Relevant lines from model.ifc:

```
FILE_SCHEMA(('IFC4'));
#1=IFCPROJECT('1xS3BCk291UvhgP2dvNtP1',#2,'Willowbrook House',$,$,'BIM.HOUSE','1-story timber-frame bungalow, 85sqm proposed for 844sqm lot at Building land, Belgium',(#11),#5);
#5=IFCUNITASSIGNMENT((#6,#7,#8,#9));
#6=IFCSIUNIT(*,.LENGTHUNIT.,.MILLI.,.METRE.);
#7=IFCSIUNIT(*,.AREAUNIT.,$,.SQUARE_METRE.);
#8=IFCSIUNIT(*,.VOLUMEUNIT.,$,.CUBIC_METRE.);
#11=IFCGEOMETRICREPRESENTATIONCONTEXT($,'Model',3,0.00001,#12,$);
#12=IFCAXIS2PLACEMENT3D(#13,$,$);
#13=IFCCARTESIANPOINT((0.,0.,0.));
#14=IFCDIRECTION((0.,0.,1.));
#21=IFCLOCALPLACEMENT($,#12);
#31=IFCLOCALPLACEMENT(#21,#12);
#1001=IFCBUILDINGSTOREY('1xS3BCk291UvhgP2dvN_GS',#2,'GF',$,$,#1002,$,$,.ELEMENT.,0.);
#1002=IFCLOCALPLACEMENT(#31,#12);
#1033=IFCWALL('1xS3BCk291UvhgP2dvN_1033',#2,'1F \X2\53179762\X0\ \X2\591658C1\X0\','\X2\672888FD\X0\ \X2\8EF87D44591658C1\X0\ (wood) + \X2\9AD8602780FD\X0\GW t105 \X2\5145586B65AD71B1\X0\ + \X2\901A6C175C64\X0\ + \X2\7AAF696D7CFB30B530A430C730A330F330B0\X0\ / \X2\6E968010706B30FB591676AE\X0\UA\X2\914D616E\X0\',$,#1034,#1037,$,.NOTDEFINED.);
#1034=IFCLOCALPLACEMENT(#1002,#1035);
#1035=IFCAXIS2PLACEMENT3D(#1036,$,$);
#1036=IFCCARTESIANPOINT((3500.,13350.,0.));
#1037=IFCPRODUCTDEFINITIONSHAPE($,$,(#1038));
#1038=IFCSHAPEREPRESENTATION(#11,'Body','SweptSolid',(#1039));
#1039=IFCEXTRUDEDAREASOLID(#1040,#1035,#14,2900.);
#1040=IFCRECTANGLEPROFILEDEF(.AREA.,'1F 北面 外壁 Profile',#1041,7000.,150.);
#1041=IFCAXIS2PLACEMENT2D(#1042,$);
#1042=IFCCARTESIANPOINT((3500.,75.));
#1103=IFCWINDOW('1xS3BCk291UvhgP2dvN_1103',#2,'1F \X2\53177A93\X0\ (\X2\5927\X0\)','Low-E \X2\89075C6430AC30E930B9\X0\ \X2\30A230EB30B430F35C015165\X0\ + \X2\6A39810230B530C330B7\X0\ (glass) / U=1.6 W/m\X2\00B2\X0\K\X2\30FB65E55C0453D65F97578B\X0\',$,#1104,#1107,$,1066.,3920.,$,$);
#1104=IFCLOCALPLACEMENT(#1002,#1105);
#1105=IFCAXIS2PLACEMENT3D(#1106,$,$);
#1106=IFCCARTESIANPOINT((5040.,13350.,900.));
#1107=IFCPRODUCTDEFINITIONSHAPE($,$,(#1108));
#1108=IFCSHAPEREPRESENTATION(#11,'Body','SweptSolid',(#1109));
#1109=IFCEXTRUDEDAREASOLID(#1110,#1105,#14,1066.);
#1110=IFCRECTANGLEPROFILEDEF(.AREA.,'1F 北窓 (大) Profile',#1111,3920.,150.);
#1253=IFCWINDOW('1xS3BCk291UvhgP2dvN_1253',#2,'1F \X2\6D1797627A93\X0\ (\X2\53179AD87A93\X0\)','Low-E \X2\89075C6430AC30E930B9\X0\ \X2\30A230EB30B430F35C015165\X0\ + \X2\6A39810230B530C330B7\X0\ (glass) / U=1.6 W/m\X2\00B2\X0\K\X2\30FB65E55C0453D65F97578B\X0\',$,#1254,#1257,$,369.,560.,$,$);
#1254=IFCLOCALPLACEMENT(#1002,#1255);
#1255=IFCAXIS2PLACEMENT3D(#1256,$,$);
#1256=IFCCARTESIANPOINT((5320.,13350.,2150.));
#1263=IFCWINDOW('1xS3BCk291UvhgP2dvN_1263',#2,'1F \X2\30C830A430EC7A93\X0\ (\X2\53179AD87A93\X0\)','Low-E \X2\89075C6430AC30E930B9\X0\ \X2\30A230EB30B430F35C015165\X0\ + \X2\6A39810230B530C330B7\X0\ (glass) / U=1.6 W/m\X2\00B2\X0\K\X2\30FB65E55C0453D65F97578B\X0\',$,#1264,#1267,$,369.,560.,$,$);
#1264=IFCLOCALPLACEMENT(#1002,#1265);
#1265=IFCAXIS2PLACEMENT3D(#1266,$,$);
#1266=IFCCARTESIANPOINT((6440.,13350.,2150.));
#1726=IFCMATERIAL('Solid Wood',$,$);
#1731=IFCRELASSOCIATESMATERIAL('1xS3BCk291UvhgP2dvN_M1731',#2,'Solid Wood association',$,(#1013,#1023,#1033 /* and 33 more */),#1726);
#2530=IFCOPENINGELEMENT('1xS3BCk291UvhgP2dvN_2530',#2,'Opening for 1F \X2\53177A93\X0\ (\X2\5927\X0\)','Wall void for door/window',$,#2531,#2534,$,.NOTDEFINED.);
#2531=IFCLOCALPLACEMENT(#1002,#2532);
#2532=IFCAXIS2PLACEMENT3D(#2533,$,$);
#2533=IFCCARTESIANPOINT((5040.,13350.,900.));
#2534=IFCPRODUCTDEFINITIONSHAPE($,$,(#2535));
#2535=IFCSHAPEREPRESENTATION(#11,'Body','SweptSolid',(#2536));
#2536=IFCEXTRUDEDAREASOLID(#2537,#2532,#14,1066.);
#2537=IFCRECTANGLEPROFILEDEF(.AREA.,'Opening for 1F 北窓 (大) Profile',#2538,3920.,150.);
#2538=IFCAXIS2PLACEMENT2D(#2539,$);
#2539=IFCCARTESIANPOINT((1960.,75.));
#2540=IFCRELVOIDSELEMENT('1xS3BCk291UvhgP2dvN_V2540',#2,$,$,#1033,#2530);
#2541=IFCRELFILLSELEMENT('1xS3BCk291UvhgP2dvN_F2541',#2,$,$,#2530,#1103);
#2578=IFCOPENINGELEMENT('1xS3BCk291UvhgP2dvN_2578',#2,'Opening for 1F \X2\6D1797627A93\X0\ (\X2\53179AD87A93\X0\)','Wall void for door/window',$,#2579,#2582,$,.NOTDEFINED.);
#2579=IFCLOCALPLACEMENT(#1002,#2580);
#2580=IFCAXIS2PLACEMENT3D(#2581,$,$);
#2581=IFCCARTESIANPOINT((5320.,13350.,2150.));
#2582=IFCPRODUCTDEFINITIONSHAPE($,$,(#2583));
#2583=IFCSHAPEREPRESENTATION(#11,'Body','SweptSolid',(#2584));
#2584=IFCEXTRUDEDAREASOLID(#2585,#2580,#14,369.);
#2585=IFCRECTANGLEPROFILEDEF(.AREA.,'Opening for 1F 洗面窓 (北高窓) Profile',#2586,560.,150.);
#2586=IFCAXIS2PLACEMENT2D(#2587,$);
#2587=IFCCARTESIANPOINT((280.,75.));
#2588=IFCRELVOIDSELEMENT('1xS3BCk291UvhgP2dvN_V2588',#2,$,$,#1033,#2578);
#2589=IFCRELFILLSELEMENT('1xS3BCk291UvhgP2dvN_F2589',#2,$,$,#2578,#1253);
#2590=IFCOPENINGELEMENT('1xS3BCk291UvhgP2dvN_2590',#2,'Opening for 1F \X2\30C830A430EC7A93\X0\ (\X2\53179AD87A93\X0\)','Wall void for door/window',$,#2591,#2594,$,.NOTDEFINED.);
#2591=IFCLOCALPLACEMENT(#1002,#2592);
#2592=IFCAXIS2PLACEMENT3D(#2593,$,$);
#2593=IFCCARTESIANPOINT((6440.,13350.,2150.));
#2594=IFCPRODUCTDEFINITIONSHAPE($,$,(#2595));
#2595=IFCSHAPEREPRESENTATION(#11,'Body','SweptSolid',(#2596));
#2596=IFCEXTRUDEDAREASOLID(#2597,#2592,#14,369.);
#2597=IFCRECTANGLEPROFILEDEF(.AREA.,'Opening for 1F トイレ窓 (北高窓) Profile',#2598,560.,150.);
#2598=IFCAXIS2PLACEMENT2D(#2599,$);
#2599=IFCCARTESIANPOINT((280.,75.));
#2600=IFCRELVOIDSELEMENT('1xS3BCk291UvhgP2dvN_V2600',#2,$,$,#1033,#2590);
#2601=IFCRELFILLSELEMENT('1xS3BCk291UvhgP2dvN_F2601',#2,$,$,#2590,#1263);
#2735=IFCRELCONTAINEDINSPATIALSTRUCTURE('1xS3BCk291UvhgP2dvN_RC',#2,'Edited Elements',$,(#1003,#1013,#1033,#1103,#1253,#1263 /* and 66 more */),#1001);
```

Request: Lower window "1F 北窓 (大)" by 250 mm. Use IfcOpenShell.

```python
import numpy as np
import ifcopenshell
import ifcopenshell.api.geometry
import ifcopenshell.util.placement
import ifcopenshell.util.unit

model = ifcopenshell.open("model.ifc")
unit_scale = ifcopenshell.util.unit.calculate_unit_scale(model)

window = model.by_guid("1xS3BCk291UvhgP2dvN_1103")
opening = window.FillsVoids[0].RelatingOpeningElement
dz = -0.25 / unit_scale

shift = np.array([0.0, 0.0, dz])
# The window is not placed relative to its opening, so move both.
for product in (opening, window):
    matrix = ifcopenshell.util.placement.get_local_placement(product.ObjectPlacement)
    matrix[:3, 3] += shift
    ifcopenshell.api.geometry.edit_object_placement(model, product=product, matrix=matrix, is_si=False)

print(f"moved by {dz * unit_scale:+.3f} m")

model.write("model_edited.ifc")
```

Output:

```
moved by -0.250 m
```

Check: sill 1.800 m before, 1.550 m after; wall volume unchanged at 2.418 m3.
